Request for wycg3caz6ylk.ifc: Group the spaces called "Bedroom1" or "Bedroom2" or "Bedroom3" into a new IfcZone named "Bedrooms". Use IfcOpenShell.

First a look at what the model holds.

```python
import ifcopenshell

model = ifcopenshell.open("wycg3caz6ylk.ifc")
print(model.schema)
seen = {}
for space in model.by_type("IfcSpace"):
    seen[space.Name] = seen.get(space.Name, 0) + 1
for name, count in sorted(seen.items(), key=str):
    print(count, "x", name)
print("zones:", [z.Name for z in model.by_type("IfcZone")][:20])
```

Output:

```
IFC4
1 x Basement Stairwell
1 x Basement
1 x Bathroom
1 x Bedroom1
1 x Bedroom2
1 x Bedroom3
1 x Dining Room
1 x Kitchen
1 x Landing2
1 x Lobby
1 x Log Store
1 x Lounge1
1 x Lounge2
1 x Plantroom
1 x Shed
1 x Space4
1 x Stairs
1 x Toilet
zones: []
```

```python
import ifcopenshell
import ifcopenshell.api.group
import ifcopenshell.api.root

model = ifcopenshell.open("wycg3caz6ylk.ifc")

names = {"Bedroom1", "Bedroom2", "Bedroom3"}
spaces = [s for s in model.by_type("IfcSpace") if s.Name in names]

zone = ifcopenshell.api.root.create_entity(model, ifc_class="IfcZone", name="Bedrooms")
ifcopenshell.api.group.assign_group(model, products=spaces, group=zone)
print(len(spaces), "spaces in", zone.Name)

model.write("wycg3caz6ylk_rev.ifc")
```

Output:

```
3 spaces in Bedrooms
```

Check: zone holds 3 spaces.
